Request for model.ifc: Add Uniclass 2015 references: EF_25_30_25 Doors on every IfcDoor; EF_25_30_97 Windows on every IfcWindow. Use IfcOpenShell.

First a look at what the model holds.

```python
import ifcopenshell

model = ifcopenshell.open("model.ifc")
print(model.schema)
print("classifications:", [c.Name for c in model.by_type("IfcClassification")])
for ifc_class in ("IfcDoor", "IfcRoof", "IfcStair", "IfcWall", "IfcWindow"):
    print(ifc_class, len(model.by_type(ifc_class)))
```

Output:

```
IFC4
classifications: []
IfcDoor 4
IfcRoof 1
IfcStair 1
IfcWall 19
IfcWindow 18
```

```python
import ifcopenshell
import ifcopenshell.api.classification

model = ifcopenshell.open("model.ifc")

system = ifcopenshell.api.classification.add_classification(model, classification="Uniclass 2015")

codes = {
    "IfcDoor": ("EF_25_30_25", "Doors"),
    "IfcWindow": ("EF_25_30_97", "Windows"),
}
for ifc_class, (code, name) in codes.items():
    products = model.by_type(ifc_class)
    ifcopenshell.api.classification.add_reference(
        model, products=products, classification=system, identification=code, name=name
    )
    print(code, len(products))

model.write("model_v2.ifc")
```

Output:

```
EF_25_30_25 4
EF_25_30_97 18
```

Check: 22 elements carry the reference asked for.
